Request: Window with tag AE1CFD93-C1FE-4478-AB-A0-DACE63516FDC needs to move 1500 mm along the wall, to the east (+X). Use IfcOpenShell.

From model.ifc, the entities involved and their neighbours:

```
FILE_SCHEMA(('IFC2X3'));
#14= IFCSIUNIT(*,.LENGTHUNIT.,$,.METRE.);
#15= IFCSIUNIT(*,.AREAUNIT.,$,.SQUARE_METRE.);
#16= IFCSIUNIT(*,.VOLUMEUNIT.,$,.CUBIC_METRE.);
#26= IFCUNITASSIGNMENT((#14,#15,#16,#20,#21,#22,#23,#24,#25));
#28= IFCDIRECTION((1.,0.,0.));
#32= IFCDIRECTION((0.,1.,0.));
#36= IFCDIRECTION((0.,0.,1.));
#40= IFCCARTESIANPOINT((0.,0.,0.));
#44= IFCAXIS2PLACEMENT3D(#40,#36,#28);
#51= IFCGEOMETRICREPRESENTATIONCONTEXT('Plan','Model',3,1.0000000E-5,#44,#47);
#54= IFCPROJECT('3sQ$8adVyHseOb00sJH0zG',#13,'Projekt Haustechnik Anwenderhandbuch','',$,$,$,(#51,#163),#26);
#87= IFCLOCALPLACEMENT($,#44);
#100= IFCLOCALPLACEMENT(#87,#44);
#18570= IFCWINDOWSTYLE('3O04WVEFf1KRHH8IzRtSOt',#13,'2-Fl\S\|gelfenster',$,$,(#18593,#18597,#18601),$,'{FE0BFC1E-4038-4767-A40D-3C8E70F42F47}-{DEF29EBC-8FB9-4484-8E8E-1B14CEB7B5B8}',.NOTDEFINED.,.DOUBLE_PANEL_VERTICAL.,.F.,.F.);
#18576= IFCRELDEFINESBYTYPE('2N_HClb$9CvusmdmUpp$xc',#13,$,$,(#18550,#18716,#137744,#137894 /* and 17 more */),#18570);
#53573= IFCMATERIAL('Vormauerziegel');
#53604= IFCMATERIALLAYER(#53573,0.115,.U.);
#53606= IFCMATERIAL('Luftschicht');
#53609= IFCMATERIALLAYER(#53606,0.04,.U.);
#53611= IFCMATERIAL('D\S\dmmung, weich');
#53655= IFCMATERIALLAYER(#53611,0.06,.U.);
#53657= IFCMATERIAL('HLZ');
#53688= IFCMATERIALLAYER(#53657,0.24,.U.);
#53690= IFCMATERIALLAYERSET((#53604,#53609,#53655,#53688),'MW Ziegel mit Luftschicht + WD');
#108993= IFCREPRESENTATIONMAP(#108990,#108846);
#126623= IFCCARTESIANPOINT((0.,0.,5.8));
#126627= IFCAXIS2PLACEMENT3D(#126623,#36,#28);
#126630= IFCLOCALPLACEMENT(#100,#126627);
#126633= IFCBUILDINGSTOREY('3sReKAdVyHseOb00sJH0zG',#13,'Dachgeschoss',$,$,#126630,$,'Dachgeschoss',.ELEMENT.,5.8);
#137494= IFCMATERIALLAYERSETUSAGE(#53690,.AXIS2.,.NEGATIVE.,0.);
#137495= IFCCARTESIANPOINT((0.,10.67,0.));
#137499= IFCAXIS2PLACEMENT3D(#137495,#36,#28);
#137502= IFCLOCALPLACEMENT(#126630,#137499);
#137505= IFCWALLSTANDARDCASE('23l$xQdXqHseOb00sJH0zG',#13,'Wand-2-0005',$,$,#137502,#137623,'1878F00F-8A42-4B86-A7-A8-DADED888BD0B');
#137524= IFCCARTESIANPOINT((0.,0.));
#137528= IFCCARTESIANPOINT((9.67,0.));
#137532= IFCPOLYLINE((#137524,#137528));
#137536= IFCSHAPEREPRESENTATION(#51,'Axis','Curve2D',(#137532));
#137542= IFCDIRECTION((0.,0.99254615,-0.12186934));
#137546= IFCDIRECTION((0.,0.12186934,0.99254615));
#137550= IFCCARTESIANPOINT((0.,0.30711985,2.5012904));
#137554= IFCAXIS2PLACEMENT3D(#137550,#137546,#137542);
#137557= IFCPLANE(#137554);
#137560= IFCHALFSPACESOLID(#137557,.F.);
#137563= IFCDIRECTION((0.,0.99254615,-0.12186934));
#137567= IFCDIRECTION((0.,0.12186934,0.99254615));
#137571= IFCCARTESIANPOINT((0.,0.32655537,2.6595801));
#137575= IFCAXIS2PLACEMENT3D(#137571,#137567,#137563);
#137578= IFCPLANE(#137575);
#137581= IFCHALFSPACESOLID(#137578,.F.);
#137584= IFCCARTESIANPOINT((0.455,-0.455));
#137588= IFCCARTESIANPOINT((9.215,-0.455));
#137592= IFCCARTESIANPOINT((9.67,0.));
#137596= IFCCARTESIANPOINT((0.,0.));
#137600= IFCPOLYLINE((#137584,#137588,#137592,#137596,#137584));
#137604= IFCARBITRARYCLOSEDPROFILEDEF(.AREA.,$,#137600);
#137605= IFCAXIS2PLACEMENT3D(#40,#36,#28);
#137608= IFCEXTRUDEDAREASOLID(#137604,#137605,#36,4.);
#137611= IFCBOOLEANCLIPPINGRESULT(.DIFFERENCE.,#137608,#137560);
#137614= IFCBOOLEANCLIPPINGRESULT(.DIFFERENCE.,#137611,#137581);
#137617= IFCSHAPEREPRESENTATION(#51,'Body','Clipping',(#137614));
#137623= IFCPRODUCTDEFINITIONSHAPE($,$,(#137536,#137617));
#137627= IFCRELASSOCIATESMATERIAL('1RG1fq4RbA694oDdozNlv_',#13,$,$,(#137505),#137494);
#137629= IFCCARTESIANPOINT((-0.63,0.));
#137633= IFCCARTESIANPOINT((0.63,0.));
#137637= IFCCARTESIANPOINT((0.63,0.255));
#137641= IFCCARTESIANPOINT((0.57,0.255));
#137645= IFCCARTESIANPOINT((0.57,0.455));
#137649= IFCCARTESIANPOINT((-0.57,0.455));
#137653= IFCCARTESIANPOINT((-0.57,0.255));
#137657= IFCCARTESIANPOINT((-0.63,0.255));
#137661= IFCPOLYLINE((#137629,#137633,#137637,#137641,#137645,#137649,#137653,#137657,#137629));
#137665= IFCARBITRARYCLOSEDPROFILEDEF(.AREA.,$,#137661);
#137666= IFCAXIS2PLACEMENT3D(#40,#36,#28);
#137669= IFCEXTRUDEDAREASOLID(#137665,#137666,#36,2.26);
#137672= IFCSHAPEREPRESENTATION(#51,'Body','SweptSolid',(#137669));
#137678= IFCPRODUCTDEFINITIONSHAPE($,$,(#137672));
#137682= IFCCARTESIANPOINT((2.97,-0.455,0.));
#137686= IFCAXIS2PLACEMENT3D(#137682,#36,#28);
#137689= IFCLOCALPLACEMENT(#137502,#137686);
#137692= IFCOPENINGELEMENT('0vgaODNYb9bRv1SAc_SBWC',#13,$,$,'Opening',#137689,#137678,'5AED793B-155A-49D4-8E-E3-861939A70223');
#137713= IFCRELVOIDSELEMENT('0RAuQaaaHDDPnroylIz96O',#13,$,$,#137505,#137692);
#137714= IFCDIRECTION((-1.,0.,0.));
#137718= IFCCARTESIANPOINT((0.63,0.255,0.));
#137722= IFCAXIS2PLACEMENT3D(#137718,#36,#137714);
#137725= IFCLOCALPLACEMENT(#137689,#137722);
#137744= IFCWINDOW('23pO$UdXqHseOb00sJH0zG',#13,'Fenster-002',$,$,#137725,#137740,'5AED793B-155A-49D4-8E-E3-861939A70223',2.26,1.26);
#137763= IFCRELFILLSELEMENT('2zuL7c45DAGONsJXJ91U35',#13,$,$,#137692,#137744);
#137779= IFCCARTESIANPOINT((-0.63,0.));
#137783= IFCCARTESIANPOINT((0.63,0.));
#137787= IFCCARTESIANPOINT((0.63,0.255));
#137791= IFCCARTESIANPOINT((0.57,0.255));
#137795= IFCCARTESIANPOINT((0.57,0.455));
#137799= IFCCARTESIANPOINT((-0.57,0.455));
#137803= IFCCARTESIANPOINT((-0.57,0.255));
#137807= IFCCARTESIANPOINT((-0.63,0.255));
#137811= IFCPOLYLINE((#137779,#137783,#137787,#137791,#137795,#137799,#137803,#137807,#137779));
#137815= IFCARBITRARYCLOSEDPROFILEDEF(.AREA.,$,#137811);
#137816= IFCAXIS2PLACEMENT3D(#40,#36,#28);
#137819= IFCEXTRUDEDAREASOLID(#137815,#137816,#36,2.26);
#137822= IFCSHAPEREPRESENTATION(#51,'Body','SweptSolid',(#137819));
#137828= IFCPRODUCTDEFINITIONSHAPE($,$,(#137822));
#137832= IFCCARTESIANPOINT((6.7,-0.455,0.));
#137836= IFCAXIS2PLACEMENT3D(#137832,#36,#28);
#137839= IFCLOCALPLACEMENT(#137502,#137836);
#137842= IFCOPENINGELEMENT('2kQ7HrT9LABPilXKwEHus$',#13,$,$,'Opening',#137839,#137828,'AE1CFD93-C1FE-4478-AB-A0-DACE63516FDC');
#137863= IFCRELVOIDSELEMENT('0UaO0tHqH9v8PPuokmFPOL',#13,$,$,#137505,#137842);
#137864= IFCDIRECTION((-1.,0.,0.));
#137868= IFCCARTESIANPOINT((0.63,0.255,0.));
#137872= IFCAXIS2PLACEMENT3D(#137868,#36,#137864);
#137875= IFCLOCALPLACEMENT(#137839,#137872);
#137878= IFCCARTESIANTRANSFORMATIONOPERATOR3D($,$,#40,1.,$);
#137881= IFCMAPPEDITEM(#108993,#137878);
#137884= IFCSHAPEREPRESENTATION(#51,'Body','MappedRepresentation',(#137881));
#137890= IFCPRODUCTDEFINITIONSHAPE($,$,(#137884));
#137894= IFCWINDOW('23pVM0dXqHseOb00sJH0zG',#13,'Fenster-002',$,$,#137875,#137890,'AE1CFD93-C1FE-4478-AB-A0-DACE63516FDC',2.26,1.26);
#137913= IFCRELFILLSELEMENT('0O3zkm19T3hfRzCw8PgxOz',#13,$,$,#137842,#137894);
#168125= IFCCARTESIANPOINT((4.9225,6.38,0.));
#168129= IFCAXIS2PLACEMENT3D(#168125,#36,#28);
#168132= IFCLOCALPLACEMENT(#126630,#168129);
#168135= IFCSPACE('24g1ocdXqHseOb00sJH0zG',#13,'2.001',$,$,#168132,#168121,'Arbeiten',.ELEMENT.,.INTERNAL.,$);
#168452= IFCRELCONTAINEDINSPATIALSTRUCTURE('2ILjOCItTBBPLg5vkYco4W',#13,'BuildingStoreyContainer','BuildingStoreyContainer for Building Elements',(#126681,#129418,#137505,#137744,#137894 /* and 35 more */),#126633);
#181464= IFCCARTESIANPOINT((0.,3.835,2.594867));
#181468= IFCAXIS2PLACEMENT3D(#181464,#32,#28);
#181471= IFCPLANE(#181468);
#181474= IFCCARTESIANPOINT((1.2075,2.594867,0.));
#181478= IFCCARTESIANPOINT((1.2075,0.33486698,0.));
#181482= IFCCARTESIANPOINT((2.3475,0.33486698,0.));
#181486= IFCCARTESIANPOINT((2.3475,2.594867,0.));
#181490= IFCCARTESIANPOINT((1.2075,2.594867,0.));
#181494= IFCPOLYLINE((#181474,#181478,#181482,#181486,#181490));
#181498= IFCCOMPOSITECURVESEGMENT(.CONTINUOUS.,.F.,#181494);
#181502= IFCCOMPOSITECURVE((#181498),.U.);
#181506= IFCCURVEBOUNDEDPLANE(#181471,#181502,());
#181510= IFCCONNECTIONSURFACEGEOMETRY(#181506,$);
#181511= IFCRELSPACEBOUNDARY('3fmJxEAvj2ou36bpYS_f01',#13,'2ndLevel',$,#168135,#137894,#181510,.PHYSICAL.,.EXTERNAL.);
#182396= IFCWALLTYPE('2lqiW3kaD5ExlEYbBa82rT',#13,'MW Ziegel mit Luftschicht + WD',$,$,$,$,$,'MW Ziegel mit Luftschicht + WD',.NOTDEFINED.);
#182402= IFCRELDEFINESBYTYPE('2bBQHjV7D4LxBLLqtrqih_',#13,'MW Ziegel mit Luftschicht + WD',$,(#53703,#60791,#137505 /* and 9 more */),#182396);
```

```python
import numpy as np
import ifcopenshell
import ifcopenshell.api.geometry
import ifcopenshell.util.placement
import ifcopenshell.util.unit

model = ifcopenshell.open("model.ifc")
unit_scale = ifcopenshell.util.unit.calculate_unit_scale(model)

window = model.by_guid("23pVM0dXqHseOb00sJH0zG")
opening = window.FillsVoids[0].RelatingOpeningElement
wall = opening.VoidsElements[0].RelatingBuildingElement

wall_matrix = ifcopenshell.util.placement.get_local_placement(wall.ObjectPlacement)
shift = wall_matrix[:3, 0] * 1.5 / unit_scale
before = ifcopenshell.util.placement.get_local_placement(window.ObjectPlacement)[:3, 3].copy()

# The window is placed relative to its opening, so it follows when the opening moves.
matrix = ifcopenshell.util.placement.get_local_placement(opening.ObjectPlacement)
matrix[:3, 3] += shift
ifcopenshell.api.geometry.edit_object_placement(
    model, product=opening, matrix=matrix, is_si=False, should_transform_children=True
)

# Space boundary surfaces are stored in each space's coordinates; move them too.
for rel in window.ProvidesBoundaries:
    if not rel.ConnectionGeometry:
        continue
    surface = rel.ConnectionGeometry.SurfaceOnRelatingElement.BasisSurface
    space_matrix = ifcopenshell.util.placement.get_local_placement(rel.RelatingSpace.ObjectPlacement)
    point = np.array(surface.Position.Location.Coordinates) + space_matrix[:3, :3].T @ shift
    surface.Position = model.createIfcAxis2Placement3D(
        model.createIfcCartesianPoint(point.tolist()), surface.Position.Axis, surface.Position.RefDirection
    )

after = ifcopenshell.util.placement.get_local_placement(window.ObjectPlacement)[:3, 3]
print("window moved by", (after - before).round(3) + 0.0)

model.write("model_v2.ifc")
```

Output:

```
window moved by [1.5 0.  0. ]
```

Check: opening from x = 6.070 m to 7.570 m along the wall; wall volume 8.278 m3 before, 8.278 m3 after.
